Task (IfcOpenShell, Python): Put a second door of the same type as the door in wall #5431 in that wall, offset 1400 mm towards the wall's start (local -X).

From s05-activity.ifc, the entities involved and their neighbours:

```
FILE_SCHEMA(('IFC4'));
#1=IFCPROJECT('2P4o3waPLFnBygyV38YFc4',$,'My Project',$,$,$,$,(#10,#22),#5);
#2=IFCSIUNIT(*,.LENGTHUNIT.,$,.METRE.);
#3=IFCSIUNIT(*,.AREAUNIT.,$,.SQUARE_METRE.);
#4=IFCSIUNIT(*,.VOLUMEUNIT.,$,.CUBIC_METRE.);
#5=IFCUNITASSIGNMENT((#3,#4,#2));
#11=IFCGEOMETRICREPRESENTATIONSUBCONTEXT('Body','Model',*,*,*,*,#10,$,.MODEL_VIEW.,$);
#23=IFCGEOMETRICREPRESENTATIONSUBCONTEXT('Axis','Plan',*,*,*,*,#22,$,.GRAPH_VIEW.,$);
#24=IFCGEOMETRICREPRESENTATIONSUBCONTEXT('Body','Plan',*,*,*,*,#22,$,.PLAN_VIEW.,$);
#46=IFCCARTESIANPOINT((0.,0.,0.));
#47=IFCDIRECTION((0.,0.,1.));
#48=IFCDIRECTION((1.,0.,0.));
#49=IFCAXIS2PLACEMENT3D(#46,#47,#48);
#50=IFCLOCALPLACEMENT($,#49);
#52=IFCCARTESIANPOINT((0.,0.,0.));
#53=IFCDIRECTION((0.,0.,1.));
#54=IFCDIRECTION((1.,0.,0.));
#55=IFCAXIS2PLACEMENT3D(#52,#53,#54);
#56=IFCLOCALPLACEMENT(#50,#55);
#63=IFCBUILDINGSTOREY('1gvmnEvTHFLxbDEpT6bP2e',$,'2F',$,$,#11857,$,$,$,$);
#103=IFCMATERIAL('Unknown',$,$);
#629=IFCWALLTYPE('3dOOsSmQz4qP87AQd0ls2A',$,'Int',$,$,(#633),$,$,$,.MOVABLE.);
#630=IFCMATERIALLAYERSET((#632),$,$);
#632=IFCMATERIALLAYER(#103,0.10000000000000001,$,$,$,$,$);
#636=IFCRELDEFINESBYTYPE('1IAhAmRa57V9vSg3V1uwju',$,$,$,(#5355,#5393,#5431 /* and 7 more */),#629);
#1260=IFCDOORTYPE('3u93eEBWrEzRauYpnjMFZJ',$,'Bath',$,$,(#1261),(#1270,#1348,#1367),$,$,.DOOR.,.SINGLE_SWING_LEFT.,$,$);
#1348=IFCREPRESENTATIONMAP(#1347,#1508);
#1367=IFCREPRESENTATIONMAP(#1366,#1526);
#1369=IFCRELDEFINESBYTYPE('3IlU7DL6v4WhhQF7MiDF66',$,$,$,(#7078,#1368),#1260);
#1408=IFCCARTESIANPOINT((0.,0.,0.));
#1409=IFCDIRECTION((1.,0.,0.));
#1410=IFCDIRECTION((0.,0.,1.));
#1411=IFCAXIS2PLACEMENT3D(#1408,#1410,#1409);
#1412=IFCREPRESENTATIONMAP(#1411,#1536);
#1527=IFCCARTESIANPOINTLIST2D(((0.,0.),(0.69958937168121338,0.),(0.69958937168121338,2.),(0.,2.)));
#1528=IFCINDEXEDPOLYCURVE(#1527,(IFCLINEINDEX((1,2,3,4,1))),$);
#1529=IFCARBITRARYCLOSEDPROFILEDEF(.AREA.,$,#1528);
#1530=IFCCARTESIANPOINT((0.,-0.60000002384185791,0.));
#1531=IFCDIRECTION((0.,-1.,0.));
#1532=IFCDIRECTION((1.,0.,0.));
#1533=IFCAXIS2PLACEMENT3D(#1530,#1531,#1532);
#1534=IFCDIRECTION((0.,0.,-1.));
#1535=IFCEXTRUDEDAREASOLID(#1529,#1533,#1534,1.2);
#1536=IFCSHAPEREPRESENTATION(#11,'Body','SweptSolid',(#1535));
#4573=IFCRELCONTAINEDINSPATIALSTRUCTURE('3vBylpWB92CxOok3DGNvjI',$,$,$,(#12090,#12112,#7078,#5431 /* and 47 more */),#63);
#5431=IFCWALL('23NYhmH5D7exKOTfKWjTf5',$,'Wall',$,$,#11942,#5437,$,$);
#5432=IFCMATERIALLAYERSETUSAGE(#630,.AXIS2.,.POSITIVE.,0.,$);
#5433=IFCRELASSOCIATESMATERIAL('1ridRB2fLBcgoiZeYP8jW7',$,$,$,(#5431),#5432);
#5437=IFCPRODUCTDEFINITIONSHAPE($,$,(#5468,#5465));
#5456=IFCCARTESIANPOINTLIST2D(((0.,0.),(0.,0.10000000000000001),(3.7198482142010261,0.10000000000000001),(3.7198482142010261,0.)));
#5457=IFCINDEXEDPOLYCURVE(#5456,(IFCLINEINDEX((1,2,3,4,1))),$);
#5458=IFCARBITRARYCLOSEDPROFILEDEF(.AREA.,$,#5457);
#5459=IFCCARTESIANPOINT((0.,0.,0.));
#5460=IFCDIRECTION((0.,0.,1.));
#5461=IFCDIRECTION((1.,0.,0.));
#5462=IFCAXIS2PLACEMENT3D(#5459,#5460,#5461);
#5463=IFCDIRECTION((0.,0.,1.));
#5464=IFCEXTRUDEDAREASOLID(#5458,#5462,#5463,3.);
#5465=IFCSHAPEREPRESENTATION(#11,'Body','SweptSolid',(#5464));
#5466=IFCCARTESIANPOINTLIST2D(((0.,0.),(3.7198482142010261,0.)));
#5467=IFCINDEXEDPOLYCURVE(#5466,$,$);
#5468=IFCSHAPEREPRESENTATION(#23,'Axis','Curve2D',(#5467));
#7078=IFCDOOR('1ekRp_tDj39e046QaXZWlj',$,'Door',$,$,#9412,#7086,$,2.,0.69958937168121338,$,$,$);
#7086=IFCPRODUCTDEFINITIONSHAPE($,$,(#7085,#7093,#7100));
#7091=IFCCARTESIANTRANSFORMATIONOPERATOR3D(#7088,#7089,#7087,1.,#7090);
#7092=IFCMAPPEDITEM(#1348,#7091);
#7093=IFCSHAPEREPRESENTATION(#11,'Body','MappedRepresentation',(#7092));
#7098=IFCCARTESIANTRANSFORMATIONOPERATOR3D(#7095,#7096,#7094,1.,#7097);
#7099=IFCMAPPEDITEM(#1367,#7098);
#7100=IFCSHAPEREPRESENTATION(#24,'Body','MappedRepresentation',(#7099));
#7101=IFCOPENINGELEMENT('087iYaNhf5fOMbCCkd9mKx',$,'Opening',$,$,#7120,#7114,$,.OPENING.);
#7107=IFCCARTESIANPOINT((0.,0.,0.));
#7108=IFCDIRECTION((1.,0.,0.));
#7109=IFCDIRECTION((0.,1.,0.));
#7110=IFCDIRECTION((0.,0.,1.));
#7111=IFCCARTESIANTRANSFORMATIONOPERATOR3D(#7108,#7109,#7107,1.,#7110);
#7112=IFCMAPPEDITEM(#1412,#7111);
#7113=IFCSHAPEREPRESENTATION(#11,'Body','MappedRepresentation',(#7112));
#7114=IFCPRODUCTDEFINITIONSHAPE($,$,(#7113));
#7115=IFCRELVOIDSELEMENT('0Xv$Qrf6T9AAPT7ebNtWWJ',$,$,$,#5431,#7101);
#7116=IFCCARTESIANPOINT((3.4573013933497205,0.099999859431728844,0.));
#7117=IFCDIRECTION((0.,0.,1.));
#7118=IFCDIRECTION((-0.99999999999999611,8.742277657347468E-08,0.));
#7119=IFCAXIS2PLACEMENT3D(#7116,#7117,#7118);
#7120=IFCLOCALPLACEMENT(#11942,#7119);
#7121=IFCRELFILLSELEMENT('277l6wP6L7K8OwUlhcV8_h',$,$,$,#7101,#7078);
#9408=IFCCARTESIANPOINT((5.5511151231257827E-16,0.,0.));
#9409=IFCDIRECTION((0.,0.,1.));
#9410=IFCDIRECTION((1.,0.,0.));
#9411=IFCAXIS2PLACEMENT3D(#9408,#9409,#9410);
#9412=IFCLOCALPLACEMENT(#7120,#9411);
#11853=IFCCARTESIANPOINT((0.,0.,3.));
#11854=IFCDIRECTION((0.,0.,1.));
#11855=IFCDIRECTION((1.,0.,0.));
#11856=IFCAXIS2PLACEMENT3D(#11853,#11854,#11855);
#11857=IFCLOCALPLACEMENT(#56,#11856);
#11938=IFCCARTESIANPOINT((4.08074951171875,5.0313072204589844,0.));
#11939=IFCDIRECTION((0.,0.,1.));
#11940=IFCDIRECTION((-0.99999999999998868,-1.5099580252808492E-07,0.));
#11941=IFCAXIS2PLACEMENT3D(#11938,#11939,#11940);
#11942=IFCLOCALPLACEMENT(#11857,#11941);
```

```python
import ifcopenshell
import ifcopenshell.api.feature
import ifcopenshell.api.geometry
import ifcopenshell.api.root
import ifcopenshell.geom
import ifcopenshell.util.element
import ifcopenshell.util.placement
import ifcopenshell.util.shape
import ifcopenshell.util.unit

model = ifcopenshell.open("s05-activity.ifc")
unit_scale = ifcopenshell.util.unit.calculate_unit_scale(model)
settings = ifcopenshell.geom.settings()


def volume(element):
    """Net volume in cubic metres, openings subtracted."""
    shape = ifcopenshell.geom.create_shape(settings, element)
    return ifcopenshell.util.shape.get_volume(shape.geometry)


door = model.by_guid("1ekRp_tDj39e046QaXZWlj")
opening = door.FillsVoids[0].RelatingOpeningElement
wall = opening.VoidsElements[0].RelatingBuildingElement
before = volume(wall)
shift = ifcopenshell.util.placement.get_local_placement(wall.ObjectPlacement)[:3, 0] * -1.4 / unit_scale

# copy_class copies the void relationship, type, container and properties, but no geometry.
new_opening = ifcopenshell.api.root.copy_class(model, product=opening)
new_opening.Representation = ifcopenshell.util.element.copy_deep(
    model, opening.Representation, exclude=["IfcGeometricRepresentationContext", "IfcRepresentationMap"]
)
new_door = ifcopenshell.api.root.copy_class(model, product=door)
new_door.Representation = ifcopenshell.util.element.copy_deep(
    model, door.Representation, exclude=["IfcGeometricRepresentationContext", "IfcRepresentationMap"]
)
ifcopenshell.api.feature.add_filling(model, opening=new_opening, element=new_door)

for old, new in ((opening, new_opening), (door, new_door)):
    matrix = ifcopenshell.util.placement.get_local_placement(old.ObjectPlacement)
    matrix[:3, 3] += shift
    ifcopenshell.api.geometry.edit_object_placement(model, product=new, matrix=matrix, is_si=False)

after = volume(wall)

print(f"wall volume {before:.3f} -> {after:.3f} m3")

model.write("s05-activity-out.ifc")
```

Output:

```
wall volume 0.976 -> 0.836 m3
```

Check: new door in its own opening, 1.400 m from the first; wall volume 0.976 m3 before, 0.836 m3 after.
